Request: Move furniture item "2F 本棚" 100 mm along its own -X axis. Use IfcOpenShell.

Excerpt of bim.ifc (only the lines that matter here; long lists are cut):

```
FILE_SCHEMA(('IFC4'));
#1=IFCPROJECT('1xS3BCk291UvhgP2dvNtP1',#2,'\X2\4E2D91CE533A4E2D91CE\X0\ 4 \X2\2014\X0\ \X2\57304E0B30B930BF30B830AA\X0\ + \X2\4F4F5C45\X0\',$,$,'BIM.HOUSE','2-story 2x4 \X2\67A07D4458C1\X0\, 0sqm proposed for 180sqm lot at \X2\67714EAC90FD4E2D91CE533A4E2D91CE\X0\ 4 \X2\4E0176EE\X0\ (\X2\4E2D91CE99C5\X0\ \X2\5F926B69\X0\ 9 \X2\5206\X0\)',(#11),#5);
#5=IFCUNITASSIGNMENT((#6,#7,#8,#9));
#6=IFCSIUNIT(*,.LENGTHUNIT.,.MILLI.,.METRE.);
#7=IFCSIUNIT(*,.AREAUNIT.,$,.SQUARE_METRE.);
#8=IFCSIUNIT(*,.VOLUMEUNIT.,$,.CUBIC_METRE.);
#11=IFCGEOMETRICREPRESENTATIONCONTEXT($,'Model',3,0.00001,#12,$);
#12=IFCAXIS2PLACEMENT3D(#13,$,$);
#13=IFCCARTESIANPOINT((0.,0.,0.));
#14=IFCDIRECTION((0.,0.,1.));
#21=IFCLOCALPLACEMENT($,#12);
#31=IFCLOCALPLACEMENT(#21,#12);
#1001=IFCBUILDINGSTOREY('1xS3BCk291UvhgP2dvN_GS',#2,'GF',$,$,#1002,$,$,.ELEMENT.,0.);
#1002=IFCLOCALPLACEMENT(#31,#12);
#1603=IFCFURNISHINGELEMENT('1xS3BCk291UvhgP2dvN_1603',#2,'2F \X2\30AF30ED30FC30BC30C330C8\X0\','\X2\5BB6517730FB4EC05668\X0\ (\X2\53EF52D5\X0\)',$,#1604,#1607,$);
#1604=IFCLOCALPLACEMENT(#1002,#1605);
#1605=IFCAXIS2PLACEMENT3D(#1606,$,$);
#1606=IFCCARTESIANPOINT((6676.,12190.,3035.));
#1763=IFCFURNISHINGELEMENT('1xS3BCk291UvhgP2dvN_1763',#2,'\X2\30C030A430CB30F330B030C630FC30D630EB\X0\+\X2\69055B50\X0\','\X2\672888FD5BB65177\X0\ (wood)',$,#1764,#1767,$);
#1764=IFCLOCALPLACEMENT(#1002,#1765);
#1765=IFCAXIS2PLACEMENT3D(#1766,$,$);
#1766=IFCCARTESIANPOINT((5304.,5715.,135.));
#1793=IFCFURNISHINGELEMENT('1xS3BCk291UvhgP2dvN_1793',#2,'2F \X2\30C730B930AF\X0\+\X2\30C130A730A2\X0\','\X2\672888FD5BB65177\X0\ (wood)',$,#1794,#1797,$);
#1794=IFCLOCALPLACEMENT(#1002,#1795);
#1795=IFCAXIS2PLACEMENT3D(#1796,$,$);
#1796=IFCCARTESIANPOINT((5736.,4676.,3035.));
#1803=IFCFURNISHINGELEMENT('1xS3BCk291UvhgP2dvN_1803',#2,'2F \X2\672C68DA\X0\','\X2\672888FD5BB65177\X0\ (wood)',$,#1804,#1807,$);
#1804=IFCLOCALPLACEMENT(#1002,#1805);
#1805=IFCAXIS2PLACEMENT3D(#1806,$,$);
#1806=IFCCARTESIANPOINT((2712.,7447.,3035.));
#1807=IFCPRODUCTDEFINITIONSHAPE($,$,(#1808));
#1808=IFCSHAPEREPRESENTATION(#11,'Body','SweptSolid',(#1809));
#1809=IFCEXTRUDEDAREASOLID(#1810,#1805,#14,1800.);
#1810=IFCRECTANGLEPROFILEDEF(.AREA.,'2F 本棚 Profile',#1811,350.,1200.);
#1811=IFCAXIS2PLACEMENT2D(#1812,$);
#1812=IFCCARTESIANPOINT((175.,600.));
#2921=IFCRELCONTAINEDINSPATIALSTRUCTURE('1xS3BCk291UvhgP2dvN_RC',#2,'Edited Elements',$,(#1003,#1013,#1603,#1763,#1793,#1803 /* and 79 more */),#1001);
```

```python
import ifcopenshell
import ifcopenshell.api.geometry
import ifcopenshell.util.placement
import ifcopenshell.util.unit

model = ifcopenshell.open("bim.ifc")
unit_scale = ifcopenshell.util.unit.calculate_unit_scale(model)

item = model.by_guid("1xS3BCk291UvhgP2dvN_1803")
matrix = ifcopenshell.util.placement.get_local_placement(item.ObjectPlacement)
matrix[:3, 3] -= matrix[:3, 0] * 0.1 / unit_scale
ifcopenshell.api.geometry.edit_object_placement(model, product=item, matrix=matrix, is_si=False)

print(ifcopenshell.util.placement.get_local_placement(item.ObjectPlacement).round(3) + 0.0)

model.write("bim_edited.ifc")
```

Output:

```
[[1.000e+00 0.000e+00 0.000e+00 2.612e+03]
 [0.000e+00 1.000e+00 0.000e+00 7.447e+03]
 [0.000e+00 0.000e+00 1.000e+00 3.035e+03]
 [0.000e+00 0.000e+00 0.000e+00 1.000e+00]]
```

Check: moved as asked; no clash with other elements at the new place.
